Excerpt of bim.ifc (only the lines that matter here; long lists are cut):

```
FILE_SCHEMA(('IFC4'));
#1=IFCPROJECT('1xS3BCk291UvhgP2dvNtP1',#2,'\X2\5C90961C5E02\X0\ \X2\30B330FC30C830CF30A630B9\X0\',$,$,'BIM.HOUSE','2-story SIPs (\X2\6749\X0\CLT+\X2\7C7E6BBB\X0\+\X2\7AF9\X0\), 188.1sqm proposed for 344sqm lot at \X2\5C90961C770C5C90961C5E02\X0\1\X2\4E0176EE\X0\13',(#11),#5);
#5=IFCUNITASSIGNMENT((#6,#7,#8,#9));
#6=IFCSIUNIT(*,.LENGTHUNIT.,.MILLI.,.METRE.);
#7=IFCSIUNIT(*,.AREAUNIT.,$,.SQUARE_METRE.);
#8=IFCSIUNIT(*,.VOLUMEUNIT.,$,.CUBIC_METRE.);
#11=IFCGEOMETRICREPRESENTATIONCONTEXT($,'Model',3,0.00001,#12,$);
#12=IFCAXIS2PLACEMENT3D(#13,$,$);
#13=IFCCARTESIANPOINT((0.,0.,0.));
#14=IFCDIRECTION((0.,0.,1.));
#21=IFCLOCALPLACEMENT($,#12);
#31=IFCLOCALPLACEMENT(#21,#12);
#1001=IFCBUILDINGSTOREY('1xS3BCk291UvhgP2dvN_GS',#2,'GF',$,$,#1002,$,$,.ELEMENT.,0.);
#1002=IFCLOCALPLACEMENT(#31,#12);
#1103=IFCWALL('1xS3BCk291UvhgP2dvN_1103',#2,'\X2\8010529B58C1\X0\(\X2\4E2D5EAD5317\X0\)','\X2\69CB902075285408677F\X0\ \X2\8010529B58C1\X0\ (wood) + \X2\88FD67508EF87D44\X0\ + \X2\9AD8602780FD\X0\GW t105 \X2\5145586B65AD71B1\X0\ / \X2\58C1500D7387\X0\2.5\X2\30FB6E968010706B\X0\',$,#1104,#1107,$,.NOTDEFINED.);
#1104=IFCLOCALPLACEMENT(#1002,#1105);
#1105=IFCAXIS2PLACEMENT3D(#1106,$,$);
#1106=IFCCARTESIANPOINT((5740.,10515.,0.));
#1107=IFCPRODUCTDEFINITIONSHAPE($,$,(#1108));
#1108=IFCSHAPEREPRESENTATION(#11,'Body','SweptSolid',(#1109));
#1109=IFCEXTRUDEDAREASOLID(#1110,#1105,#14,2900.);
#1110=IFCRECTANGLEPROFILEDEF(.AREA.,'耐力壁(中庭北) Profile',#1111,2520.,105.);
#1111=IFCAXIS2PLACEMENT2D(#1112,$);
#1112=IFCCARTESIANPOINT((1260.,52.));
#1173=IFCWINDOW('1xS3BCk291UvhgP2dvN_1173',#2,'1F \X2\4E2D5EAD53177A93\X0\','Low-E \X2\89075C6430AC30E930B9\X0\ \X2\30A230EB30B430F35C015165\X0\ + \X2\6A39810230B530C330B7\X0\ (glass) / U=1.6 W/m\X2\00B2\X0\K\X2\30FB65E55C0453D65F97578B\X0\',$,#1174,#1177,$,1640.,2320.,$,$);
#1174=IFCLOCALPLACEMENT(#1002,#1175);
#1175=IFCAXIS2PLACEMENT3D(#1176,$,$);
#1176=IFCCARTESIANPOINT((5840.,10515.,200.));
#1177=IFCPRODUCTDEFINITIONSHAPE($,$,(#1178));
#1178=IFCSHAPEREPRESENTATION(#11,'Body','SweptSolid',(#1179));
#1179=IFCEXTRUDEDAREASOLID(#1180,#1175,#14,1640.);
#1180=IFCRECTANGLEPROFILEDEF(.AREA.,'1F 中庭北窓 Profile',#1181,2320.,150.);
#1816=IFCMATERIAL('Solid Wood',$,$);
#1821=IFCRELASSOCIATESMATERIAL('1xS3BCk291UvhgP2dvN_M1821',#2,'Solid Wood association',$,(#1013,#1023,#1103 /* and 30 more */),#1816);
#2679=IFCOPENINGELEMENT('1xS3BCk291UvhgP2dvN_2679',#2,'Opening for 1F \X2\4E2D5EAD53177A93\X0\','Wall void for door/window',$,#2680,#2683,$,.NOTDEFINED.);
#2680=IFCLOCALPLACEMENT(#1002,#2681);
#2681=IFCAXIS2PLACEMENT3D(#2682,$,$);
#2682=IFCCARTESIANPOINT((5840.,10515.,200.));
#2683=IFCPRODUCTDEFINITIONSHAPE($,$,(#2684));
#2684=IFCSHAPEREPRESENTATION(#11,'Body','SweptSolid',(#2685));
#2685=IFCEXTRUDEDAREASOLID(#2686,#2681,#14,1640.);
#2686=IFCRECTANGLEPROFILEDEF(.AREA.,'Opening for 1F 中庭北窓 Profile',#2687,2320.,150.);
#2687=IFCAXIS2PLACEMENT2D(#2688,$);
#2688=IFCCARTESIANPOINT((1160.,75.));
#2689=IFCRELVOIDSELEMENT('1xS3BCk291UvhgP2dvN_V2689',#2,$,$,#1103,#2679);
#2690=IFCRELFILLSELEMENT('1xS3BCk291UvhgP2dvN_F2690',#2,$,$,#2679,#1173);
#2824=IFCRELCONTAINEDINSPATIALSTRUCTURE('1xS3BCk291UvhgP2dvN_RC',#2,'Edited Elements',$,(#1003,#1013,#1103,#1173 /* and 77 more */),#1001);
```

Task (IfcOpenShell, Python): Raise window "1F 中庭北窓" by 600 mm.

```python
import numpy as np
import ifcopenshell
import ifcopenshell.api.geometry
import ifcopenshell.util.placement
import ifcopenshell.util.unit

model = ifcopenshell.open("bim.ifc")
unit_scale = ifcopenshell.util.unit.calculate_unit_scale(model)

window = model.by_guid("1xS3BCk291UvhgP2dvN_1173")
opening = window.FillsVoids[0].RelatingOpeningElement
dz = 600.0

shift = np.array([0.0, 0.0, dz])
# The window is not placed relative to its opening, so move both.
for product in (opening, window):
    matrix = ifcopenshell.util.placement.get_local_placement(product.ObjectPlacement)
    matrix[:3, 3] += shift
    ifcopenshell.api.geometry.edit_object_placement(model, product=product, matrix=matrix, is_si=False)

print(f"moved by {dz * unit_scale:+.3f} m")

model.write("bim_updated.ifc")
```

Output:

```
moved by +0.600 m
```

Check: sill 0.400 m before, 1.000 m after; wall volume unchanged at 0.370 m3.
